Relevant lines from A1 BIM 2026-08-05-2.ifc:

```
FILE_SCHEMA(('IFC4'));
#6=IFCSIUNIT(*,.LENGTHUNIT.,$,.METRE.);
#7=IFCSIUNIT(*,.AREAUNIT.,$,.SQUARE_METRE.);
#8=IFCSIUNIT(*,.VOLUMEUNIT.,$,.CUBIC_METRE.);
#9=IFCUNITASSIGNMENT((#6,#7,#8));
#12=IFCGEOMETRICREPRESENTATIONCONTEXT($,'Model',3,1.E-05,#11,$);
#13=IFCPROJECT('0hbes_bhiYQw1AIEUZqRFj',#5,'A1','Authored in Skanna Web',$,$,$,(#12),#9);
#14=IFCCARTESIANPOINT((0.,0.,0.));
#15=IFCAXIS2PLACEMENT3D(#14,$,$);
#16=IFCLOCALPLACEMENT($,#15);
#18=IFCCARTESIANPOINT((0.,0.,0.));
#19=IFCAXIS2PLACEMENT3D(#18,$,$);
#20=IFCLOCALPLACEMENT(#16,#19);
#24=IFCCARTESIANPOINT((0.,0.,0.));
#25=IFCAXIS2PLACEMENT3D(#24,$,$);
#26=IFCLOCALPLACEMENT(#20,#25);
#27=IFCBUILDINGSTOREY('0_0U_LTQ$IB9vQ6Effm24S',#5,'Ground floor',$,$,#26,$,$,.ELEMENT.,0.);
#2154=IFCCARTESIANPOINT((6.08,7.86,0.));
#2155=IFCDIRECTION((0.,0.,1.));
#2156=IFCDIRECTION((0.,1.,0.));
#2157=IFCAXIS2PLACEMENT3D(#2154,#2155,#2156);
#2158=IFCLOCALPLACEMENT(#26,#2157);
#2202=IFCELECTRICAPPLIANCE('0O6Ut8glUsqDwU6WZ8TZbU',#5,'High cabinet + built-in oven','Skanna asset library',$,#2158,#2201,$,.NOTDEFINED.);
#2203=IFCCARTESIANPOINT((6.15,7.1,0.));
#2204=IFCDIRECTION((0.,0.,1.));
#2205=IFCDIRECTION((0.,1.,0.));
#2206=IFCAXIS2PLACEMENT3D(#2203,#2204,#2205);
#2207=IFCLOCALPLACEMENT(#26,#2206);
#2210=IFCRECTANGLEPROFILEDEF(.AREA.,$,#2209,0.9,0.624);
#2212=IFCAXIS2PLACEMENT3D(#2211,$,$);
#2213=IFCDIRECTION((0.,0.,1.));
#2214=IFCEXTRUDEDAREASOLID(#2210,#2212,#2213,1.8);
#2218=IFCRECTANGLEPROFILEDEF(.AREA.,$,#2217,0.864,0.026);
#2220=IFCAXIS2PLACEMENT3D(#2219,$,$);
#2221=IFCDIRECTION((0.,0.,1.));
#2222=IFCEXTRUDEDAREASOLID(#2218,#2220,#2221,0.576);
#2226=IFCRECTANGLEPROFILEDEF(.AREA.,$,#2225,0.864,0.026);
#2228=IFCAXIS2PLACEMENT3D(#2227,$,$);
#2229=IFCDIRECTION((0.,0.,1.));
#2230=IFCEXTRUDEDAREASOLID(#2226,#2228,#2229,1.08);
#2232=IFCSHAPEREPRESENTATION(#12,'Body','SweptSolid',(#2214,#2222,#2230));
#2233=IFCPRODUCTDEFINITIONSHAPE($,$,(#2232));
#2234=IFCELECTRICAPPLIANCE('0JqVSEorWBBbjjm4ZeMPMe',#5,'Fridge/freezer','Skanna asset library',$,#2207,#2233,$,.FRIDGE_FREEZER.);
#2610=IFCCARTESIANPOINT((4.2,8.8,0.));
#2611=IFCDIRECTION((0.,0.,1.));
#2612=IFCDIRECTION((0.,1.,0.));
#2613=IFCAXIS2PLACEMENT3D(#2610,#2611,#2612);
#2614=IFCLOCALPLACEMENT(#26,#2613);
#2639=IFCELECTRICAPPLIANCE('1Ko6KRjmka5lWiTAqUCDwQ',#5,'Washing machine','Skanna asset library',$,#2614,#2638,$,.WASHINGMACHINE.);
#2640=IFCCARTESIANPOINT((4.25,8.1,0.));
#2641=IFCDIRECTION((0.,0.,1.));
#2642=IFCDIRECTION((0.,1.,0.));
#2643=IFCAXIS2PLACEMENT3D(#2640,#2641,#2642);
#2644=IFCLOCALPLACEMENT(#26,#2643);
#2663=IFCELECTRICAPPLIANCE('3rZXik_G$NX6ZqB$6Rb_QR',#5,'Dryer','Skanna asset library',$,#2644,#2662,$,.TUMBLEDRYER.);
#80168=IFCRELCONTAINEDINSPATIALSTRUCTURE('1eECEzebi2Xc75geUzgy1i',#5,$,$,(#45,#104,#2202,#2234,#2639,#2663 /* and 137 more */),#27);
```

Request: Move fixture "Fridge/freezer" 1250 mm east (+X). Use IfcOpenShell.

```python
import ifcopenshell
import ifcopenshell.api.geometry
import ifcopenshell.util.placement
import ifcopenshell.util.unit

model = ifcopenshell.open("A1 BIM 2026-08-05-2.ifc")
unit_scale = ifcopenshell.util.unit.calculate_unit_scale(model)

item = model.by_guid("0JqVSEorWBBbjjm4ZeMPMe")
matrix = ifcopenshell.util.placement.get_local_placement(item.ObjectPlacement)
matrix[0, 3] += 1.25 / unit_scale
ifcopenshell.api.geometry.edit_object_placement(model, product=item, matrix=matrix, is_si=False)

print(ifcopenshell.util.placement.get_local_placement(item.ObjectPlacement).round(3) + 0.0)

model.write("A1 BIM 2026-08-05-2-out.ifc")
```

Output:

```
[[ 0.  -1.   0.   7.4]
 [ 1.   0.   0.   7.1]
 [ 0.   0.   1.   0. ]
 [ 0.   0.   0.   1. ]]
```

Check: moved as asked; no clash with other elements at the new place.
